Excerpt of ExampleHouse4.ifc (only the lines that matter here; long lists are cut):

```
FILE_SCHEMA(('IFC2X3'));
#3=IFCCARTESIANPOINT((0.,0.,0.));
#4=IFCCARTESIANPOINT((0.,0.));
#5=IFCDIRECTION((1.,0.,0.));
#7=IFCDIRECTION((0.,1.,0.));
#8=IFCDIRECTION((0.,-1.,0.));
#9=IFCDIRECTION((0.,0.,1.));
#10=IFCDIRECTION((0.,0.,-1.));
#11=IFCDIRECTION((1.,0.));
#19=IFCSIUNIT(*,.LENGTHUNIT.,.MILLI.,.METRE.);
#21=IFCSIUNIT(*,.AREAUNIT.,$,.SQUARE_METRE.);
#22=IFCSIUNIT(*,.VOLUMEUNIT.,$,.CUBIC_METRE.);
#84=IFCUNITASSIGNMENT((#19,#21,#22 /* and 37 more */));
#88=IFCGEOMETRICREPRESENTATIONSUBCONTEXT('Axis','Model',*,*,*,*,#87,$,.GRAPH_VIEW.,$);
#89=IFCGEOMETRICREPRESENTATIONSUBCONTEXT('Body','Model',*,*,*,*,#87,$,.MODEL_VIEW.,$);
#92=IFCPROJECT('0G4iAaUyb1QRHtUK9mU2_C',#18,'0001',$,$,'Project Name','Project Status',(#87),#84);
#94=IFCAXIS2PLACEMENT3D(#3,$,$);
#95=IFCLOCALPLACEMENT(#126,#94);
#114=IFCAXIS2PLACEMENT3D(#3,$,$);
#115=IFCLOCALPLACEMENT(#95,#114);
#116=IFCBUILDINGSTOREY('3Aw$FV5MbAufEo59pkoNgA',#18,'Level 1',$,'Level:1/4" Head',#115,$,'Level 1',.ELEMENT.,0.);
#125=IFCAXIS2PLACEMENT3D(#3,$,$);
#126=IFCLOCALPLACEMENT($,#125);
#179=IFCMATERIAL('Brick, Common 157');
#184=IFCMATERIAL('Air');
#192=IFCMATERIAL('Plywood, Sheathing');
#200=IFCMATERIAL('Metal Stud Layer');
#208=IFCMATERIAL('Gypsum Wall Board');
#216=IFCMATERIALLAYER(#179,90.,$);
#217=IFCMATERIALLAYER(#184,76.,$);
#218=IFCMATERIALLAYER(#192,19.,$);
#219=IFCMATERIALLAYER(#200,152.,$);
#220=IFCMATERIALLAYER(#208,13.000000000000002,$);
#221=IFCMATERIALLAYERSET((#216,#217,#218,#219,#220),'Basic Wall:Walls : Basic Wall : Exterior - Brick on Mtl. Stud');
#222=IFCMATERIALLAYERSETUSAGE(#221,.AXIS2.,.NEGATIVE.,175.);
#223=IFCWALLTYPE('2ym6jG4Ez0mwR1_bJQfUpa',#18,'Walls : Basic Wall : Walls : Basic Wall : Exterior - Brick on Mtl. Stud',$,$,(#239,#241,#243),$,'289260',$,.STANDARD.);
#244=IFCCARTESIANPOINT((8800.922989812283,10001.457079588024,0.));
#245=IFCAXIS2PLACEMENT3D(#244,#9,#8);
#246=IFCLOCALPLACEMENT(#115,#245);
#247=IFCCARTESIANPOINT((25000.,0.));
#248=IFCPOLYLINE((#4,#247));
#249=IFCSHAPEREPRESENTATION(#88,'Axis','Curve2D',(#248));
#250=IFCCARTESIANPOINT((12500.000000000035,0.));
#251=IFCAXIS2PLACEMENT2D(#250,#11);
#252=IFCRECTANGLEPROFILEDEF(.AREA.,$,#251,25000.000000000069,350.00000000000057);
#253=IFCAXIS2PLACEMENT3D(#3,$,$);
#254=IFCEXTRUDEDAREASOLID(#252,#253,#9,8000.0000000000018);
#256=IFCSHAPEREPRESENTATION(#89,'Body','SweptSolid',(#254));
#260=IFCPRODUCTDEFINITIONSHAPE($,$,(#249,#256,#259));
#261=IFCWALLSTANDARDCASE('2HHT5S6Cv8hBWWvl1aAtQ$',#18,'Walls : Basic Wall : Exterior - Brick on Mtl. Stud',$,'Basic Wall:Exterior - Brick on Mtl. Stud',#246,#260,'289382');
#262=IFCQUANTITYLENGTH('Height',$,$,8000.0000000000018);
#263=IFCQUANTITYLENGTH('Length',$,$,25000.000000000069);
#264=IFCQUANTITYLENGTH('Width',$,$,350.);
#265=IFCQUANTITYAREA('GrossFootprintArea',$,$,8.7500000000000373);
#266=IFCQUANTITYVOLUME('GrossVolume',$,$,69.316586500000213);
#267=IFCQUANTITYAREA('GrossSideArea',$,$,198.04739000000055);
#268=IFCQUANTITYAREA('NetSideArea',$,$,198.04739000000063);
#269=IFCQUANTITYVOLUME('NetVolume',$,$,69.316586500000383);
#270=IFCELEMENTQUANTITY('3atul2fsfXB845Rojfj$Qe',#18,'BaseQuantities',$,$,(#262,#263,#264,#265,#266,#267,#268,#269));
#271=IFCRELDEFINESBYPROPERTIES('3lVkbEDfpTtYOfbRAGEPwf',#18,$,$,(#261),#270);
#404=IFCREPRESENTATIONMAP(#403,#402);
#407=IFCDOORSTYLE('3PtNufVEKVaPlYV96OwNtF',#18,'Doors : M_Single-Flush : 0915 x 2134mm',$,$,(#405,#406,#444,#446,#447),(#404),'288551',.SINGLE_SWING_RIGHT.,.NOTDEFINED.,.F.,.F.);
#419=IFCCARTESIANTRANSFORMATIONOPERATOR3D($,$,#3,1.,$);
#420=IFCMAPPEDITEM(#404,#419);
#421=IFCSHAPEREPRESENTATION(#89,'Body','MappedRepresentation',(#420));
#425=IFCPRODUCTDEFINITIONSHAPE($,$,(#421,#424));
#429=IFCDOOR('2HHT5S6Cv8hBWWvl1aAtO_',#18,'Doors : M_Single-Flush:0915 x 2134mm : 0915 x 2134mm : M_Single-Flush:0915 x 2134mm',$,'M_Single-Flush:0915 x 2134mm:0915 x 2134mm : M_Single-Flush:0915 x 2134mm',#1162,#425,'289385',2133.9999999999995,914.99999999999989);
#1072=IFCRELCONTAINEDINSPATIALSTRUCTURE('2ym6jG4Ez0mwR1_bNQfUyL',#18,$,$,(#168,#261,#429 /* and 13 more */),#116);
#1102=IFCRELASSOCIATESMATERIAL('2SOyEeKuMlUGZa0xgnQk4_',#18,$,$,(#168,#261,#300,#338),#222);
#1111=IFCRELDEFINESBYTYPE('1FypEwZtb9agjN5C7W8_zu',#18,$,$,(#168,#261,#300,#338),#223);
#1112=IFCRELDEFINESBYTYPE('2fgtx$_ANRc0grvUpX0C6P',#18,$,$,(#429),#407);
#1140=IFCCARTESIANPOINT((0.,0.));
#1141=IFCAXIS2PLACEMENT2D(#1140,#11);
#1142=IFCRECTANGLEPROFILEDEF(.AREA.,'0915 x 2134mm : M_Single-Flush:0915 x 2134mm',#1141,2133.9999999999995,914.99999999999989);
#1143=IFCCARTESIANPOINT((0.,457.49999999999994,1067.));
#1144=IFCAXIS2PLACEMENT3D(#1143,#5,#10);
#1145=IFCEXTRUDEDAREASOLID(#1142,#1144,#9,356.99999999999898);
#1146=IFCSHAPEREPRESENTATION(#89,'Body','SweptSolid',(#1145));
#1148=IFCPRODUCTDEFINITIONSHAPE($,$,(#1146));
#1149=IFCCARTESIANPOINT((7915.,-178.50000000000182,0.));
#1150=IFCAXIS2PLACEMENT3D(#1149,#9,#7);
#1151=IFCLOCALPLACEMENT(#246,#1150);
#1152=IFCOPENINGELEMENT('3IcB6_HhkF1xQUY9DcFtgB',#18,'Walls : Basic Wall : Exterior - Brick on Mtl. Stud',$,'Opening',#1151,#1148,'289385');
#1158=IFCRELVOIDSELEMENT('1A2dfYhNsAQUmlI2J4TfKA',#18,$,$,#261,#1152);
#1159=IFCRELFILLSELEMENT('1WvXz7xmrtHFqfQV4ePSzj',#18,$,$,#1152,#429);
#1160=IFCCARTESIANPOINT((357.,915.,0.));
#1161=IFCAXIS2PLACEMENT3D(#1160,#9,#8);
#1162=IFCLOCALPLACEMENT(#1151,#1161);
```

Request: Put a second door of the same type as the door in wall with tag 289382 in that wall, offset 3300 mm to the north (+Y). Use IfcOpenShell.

```python
import ifcopenshell
import ifcopenshell.api.feature
import ifcopenshell.api.geometry
import ifcopenshell.api.pset
import ifcopenshell.api.root
import ifcopenshell.geom
import ifcopenshell.util.element
import ifcopenshell.util.placement
import ifcopenshell.util.shape
import ifcopenshell.util.unit

model = ifcopenshell.open("ExampleHouse4.ifc")
area_scale = ifcopenshell.util.unit.calculate_unit_scale(model, "AREAUNIT")
volume_scale = ifcopenshell.util.unit.calculate_unit_scale(model, "VOLUMEUNIT")
settings = ifcopenshell.geom.settings()


def volume(element):
    """Net volume in cubic metres, openings subtracted."""
    shape = ifcopenshell.geom.create_shape(settings, element)
    return ifcopenshell.util.shape.get_volume(shape.geometry)


def reuse_history(source, copy):
    """copy_class also copies each property set's owner history, people and application; keep the originals."""
    for rel in copy.IsDefinedBy:
        if rel.is_a("IfcRelDefinesByProperties") and (history := rel.RelatingPropertyDefinition.OwnerHistory):
            rel.RelatingPropertyDefinition.OwnerHistory = source.OwnerHistory
            ifcopenshell.util.element.remove_deep2(model, history)


door = model.by_guid("2HHT5S6Cv8hBWWvl1aAtO_")
opening = door.FillsVoids[0].RelatingOpeningElement
wall = opening.VoidsElements[0].RelatingBuildingElement
before = volume(wall)
shift = ifcopenshell.util.placement.get_local_placement(wall.ObjectPlacement)[:3, 0] * -3300.0

# copy_class copies the void relationship, type, container and properties, but no geometry.
new_opening = ifcopenshell.api.root.copy_class(model, product=opening)
new_opening.Representation = ifcopenshell.util.element.copy_deep(
    model, opening.Representation, exclude=["IfcGeometricRepresentationContext", "IfcRepresentationMap"]
)
new_opening.Tag = None
reuse_history(opening, new_opening)
new_door = ifcopenshell.api.root.copy_class(model, product=door)
new_door.Representation = ifcopenshell.util.element.copy_deep(
    model, door.Representation, exclude=["IfcGeometricRepresentationContext", "IfcRepresentationMap"]
)
new_door.Tag = None
reuse_history(door, new_door)
fills = ifcopenshell.api.feature.add_filling(model, opening=new_opening, element=new_door)
fills.OwnerHistory = new_door.OwnerHistory  # required in IFC2X3

for old, new in ((opening, new_opening), (door, new_door)):
    matrix = ifcopenshell.util.placement.get_local_placement(old.ObjectPlacement)
    matrix[:3, 3] += shift
    ifcopenshell.api.geometry.edit_object_placement(model, product=new, matrix=matrix, is_si=False)

after = volume(wall)
thickness = 0.35  # wall thickness in metres

# Update the wall's stored quantities.
qto = model.by_id(ifcopenshell.util.element.get_pset(wall, "BaseQuantities", should_inherit=False)["id"])
ifcopenshell.api.pset.edit_qto(model, qto=qto, properties={
    "NetSideArea": after / thickness / area_scale,
    "NetVolume": after / volume_scale,
})

print(f"wall volume {before:.3f} -> {after:.3f} m3")

model.write("ExampleHouse4_rev.ifc")
```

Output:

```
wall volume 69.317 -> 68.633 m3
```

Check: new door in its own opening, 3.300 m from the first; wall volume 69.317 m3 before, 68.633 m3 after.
